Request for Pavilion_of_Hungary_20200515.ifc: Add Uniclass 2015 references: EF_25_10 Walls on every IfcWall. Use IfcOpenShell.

First a look at what the model holds.

```python
import ifcopenshell

model = ifcopenshell.open("Pavilion_of_Hungary_20200515.ifc")
print(model.schema)
print("classifications:", [c.Name for c in model.by_type("IfcClassification")])
for ifc_class in ("IfcDoor", "IfcRoof", "IfcStair", "IfcWall", "IfcWindow"):
    print(ifc_class, len(model.by_type(ifc_class)))
```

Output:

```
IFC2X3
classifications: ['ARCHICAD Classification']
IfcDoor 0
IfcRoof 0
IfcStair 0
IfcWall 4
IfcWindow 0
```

```python
import ifcopenshell
import ifcopenshell.api.classification

model = ifcopenshell.open("Pavilion_of_Hungary_20200515.ifc")

# IFC2X3 requires Source and Edition and has no link from the project to the system.
system = model.create_entity("IfcClassification", Source="NBS", Edition="2015", Name="Uniclass 2015")

codes = {
    "IfcWall": ("EF_25_10", "Walls"),
}
for ifc_class, (code, name) in codes.items():
    products = model.by_type(ifc_class)
    ifcopenshell.api.classification.add_reference(
        model, products=products, classification=system, identification=code, name=name
    )
    print(code, len(products))

model.write("Pavilion_of_Hungary_20200515_rev.ifc")
```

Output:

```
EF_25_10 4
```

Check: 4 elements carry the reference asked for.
